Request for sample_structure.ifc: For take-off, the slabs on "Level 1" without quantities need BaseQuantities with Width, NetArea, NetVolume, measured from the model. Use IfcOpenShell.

First a look at what the model holds.

```python
import ifcopenshell
import ifcopenshell.util.element
import ifcopenshell.util.unit

model = ifcopenshell.open("sample_structure.ifc")
print(model.schema)
for unit_type in ("LENGTHUNIT", "AREAUNIT", "VOLUMEUNIT"):
    print(unit_type, ifcopenshell.util.unit.calculate_unit_scale(model, unit_type))
storey = next(s for s in model.by_type("IfcBuildingStorey") if s.Name == "Level 1")
slabs = [e for e in ifcopenshell.util.element.get_decomposition(storey) if e.is_a("IfcSlab")]
for e in sorted(slabs, key=lambda e: e.id()):
    print(e.id(), e.is_a(), e.Name, list(ifcopenshell.util.element.get_psets(e, qtos_only=True)), sep=" | ")
```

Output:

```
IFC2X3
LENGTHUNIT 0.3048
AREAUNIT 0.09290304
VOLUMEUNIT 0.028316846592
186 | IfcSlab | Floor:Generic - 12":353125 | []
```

```python
import ifcopenshell
import ifcopenshell.api.pset
import ifcopenshell.geom
import ifcopenshell.util.element
import ifcopenshell.util.shape
import ifcopenshell.util.unit

model = ifcopenshell.open("sample_structure.ifc")
unit_scale = ifcopenshell.util.unit.calculate_unit_scale(model)
area_scale = ifcopenshell.util.unit.calculate_unit_scale(model, "AREAUNIT")
volume_scale = ifcopenshell.util.unit.calculate_unit_scale(model, "VOLUMEUNIT")
settings = ifcopenshell.geom.settings()

storey = next(s for s in model.by_type("IfcBuildingStorey") if s.Name == "Level 1")
slabs = [e for e in ifcopenshell.util.element.get_decomposition(storey) if e.is_a("IfcSlab")]

for e in sorted(slabs, key=lambda e: e.id()):
    if ifcopenshell.util.element.get_psets(e, qtos_only=True, should_inherit=False):
        continue
    # Geometry comes back in metres, in the element's own axes.
    shape = ifcopenshell.geom.create_shape(settings, e)
    values = {
        "Width": ifcopenshell.util.shape.get_z(shape.geometry) / unit_scale,
        "NetArea": ifcopenshell.util.shape.get_footprint_area(shape.geometry) / area_scale,
        "NetVolume": ifcopenshell.util.shape.get_volume(shape.geometry) / volume_scale,
    }
    qto = ifcopenshell.api.pset.add_qto(model, product=e, name="BaseQuantities")
    ifcopenshell.api.pset.edit_qto(model, qto=qto, properties=values)
    print(e.id(), {k: round(v, 3) for k, v in values.items()})

model.write("sample_structure_updated.ifc")
```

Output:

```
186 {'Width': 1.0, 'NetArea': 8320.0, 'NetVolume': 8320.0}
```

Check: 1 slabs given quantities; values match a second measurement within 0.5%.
